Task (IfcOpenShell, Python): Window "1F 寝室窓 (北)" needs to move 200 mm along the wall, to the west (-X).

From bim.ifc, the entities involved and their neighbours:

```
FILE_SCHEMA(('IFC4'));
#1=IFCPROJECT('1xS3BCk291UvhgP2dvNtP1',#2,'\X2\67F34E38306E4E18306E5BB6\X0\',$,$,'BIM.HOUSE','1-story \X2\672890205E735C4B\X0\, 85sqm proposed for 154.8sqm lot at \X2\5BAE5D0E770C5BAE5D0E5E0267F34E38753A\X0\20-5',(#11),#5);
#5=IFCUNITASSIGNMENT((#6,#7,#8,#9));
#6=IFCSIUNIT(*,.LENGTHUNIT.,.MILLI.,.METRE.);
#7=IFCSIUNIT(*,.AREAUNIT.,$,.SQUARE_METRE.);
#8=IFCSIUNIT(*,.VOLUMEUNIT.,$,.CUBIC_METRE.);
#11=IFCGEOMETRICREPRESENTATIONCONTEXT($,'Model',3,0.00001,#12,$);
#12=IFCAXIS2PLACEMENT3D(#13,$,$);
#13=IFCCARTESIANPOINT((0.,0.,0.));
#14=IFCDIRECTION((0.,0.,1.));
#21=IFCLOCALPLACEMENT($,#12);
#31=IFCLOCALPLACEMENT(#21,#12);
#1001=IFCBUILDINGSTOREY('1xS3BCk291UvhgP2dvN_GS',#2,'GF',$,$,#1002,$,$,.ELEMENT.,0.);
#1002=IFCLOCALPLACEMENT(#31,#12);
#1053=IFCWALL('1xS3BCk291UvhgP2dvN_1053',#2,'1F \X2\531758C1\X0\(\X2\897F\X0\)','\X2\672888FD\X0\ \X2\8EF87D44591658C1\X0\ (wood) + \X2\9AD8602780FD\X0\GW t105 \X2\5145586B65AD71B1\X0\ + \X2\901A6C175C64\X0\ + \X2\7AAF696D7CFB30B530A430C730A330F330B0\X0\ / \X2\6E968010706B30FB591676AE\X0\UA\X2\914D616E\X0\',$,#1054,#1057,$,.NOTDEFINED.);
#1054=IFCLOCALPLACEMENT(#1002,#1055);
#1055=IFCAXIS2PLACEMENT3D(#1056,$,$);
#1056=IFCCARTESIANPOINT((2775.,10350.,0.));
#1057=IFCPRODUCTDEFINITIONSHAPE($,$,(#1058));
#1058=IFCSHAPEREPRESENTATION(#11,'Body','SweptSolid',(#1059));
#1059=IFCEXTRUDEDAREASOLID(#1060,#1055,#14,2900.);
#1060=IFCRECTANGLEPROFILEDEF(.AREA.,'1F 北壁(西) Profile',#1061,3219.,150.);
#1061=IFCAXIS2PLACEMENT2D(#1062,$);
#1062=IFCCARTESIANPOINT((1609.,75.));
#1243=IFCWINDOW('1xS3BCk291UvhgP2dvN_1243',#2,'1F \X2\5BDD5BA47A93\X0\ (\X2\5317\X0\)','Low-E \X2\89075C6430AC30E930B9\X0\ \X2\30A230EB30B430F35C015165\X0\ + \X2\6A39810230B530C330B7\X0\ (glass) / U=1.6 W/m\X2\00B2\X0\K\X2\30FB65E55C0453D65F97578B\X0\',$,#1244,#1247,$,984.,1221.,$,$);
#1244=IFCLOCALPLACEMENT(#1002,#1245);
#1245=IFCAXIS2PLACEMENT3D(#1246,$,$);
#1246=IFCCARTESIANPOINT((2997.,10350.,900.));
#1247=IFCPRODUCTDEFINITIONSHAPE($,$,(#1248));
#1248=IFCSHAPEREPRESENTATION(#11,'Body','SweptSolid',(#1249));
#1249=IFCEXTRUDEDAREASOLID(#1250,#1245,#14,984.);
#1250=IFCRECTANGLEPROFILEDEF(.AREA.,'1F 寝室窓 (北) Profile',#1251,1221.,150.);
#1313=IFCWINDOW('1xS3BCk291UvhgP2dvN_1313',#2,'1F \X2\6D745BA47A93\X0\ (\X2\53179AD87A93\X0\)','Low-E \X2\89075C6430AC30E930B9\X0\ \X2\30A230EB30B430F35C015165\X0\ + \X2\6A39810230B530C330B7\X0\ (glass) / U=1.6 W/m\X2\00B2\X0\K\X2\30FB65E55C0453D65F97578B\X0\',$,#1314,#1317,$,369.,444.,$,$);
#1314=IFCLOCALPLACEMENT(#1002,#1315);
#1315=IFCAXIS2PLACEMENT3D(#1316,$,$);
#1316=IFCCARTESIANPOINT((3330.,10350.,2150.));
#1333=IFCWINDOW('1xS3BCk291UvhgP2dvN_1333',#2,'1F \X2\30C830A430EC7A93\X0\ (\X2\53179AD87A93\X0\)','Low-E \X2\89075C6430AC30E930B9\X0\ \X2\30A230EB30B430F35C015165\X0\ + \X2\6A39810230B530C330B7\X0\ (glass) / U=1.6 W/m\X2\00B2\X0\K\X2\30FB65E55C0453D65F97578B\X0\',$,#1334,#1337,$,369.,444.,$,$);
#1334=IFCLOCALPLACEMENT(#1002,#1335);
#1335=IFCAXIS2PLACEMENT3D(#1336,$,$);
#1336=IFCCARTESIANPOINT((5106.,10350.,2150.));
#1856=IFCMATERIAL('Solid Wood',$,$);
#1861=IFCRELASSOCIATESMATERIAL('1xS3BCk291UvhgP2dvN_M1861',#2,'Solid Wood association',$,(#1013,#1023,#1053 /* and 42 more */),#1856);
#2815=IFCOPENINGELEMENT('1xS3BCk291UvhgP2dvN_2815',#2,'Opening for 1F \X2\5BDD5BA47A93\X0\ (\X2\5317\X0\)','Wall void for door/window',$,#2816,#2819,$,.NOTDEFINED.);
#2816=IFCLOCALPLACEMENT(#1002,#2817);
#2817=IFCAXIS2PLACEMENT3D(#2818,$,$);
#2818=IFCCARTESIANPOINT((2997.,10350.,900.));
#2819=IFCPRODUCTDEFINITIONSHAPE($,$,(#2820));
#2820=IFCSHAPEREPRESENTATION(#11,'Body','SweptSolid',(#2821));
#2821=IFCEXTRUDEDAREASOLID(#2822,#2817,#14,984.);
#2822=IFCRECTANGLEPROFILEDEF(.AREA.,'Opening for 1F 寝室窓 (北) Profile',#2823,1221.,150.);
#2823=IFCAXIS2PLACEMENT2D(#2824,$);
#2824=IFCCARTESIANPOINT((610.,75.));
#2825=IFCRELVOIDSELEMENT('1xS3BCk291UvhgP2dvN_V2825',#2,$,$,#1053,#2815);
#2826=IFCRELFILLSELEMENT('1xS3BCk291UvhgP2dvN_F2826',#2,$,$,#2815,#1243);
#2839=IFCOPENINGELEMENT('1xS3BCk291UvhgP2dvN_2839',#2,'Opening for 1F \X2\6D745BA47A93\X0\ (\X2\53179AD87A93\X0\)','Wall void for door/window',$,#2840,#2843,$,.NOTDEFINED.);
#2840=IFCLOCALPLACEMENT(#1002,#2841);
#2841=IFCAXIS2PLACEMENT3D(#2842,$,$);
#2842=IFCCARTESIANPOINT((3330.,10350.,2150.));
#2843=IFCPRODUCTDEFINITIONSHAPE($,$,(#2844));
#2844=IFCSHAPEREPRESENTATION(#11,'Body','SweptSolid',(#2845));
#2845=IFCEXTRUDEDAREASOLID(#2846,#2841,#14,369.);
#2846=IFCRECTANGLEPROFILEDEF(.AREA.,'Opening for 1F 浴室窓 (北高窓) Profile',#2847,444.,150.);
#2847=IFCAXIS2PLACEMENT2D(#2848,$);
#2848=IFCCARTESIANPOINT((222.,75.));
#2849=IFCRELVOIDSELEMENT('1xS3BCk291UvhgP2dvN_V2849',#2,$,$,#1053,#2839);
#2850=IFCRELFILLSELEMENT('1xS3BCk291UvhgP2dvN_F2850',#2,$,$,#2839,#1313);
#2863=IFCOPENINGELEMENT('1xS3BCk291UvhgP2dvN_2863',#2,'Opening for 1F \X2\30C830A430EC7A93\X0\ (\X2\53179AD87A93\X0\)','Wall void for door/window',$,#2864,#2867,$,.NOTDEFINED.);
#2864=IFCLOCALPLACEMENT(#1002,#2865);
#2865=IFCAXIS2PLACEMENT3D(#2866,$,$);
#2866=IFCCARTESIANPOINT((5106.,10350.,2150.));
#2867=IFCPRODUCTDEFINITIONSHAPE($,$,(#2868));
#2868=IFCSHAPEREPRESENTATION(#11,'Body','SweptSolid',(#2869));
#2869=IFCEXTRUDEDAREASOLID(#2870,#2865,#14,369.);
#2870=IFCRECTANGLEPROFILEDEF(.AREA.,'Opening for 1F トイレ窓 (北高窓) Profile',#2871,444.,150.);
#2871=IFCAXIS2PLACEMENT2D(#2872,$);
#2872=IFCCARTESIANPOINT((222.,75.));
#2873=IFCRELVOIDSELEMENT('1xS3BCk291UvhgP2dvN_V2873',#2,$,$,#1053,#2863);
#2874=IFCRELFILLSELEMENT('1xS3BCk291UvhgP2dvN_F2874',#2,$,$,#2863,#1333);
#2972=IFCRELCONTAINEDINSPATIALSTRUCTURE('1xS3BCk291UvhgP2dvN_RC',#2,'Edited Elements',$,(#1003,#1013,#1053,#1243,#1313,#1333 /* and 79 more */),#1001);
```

```python
import ifcopenshell
import ifcopenshell.api.geometry
import ifcopenshell.util.placement
import ifcopenshell.util.unit

model = ifcopenshell.open("bim.ifc")
unit_scale = ifcopenshell.util.unit.calculate_unit_scale(model)

window = model.by_guid("1xS3BCk291UvhgP2dvN_1243")
opening = window.FillsVoids[0].RelatingOpeningElement
wall = opening.VoidsElements[0].RelatingBuildingElement

wall_matrix = ifcopenshell.util.placement.get_local_placement(wall.ObjectPlacement)
shift = wall_matrix[:3, 0] * -0.2 / unit_scale
before = ifcopenshell.util.placement.get_local_placement(window.ObjectPlacement)[:3, 3].copy()

# The window is not placed relative to its opening, so move both.
for product in (opening, window):
    matrix = ifcopenshell.util.placement.get_local_placement(product.ObjectPlacement)
    matrix[:3, 3] += shift
    ifcopenshell.api.geometry.edit_object_placement(model, product=product, matrix=matrix, is_si=False)

after = ifcopenshell.util.placement.get_local_placement(window.ObjectPlacement)[:3, 3]
print("window moved by", (after - before).round(3) + 0.0)

model.write("bim_updated.ifc")
```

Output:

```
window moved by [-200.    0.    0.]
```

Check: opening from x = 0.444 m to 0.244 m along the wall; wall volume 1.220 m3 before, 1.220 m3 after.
